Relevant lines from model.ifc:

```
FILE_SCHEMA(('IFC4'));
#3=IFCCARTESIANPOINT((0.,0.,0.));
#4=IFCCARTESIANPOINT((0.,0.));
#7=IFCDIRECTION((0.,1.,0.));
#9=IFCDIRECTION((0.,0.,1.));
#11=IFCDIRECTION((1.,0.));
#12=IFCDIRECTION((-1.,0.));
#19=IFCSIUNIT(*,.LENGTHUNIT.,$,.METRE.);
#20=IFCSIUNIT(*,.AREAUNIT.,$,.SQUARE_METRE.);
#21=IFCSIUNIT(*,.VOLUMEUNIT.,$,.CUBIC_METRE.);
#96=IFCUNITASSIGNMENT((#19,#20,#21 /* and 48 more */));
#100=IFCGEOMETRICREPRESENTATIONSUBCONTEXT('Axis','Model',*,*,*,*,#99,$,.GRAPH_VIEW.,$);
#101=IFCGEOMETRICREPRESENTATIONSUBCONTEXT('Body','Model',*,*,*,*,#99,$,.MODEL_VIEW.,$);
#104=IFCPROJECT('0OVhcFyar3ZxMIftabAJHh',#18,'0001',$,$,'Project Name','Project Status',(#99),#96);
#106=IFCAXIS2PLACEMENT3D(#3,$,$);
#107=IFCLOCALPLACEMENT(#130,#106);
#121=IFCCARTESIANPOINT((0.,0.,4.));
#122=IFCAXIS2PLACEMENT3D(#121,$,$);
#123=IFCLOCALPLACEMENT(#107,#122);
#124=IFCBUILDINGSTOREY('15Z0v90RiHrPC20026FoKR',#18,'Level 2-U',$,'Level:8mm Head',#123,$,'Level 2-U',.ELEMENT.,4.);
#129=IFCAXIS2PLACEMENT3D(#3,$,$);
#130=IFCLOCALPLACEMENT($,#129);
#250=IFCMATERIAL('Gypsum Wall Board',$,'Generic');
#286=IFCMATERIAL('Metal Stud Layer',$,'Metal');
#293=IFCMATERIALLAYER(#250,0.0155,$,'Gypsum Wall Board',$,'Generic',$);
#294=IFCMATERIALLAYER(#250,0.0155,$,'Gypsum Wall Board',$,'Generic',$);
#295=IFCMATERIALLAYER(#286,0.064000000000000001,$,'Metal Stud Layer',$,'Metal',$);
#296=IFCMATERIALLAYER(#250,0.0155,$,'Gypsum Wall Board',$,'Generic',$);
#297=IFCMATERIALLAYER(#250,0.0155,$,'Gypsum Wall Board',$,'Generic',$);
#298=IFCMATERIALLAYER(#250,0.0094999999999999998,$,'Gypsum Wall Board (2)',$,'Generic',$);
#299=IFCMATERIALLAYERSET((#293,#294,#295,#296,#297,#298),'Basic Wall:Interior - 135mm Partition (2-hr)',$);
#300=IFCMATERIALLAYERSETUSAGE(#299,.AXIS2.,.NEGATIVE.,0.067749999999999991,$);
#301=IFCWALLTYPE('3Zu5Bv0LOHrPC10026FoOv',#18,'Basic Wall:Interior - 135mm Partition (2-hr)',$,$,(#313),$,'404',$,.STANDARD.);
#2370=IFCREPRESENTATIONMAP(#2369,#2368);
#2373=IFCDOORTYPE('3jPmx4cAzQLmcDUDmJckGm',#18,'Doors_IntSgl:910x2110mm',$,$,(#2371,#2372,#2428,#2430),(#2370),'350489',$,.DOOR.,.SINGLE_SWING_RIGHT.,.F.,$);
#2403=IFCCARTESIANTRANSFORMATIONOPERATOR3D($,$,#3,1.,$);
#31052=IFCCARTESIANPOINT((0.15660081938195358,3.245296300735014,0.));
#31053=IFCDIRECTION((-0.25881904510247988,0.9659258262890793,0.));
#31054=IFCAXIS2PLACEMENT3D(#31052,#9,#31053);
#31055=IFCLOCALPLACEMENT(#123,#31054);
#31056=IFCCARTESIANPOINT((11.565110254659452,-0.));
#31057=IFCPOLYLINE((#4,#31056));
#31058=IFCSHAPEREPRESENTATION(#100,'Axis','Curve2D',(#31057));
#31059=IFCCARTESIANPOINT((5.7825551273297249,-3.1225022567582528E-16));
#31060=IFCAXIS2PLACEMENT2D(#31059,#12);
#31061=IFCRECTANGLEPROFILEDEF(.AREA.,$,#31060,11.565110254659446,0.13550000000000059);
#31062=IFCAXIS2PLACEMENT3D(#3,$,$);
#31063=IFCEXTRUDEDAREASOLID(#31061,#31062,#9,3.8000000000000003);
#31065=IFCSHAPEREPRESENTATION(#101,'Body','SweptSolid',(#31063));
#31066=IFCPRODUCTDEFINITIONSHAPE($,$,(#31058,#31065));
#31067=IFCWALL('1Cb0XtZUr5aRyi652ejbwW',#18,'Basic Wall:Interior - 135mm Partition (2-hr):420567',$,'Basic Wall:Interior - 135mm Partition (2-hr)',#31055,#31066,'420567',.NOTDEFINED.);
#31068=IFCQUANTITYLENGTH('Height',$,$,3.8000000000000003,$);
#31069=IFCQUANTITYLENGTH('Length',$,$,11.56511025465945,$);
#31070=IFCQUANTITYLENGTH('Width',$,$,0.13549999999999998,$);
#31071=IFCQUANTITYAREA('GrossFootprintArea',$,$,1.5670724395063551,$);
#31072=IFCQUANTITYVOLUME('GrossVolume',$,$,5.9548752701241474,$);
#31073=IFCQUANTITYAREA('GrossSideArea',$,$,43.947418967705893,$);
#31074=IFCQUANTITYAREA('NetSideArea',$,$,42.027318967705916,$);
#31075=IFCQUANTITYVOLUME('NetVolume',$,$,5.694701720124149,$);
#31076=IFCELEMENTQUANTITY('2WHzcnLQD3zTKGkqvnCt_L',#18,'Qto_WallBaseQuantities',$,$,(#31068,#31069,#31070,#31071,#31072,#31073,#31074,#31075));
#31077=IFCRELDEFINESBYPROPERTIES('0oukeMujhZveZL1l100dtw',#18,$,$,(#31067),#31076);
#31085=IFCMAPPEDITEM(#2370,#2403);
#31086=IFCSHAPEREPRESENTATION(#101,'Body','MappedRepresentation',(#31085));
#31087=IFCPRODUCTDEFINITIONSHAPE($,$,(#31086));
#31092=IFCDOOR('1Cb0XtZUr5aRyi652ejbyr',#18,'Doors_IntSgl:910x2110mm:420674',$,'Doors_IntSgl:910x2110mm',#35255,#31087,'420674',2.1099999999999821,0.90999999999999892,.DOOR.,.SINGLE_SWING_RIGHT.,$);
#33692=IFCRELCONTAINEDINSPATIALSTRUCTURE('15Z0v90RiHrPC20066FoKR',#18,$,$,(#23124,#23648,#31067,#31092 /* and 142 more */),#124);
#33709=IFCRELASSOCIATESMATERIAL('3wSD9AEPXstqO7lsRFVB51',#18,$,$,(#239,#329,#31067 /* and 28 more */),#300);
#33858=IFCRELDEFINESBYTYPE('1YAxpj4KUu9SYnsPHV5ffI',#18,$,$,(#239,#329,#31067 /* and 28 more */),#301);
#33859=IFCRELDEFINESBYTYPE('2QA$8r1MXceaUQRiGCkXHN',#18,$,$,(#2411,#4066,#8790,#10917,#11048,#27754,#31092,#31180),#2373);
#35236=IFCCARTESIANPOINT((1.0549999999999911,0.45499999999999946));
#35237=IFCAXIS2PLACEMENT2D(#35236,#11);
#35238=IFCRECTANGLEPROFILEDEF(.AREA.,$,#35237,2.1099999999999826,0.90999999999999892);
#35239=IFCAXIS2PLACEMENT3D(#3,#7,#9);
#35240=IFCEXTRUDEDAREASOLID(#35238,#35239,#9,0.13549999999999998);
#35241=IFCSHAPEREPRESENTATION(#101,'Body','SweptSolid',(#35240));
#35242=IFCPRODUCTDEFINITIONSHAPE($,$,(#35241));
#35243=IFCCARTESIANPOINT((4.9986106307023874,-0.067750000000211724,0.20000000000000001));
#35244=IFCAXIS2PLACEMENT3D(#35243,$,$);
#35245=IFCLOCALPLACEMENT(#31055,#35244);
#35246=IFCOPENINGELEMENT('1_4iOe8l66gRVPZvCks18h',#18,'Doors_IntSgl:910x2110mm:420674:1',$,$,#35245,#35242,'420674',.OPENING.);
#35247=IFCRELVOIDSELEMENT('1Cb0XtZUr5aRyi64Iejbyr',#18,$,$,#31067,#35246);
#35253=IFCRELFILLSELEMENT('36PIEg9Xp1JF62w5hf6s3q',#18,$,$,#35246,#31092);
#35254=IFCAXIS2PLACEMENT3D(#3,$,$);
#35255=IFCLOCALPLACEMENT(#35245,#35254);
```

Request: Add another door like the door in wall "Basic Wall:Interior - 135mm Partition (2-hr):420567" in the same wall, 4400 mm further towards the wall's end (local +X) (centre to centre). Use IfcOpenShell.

```python
import ifcopenshell
import ifcopenshell.api.feature
import ifcopenshell.api.geometry
import ifcopenshell.api.pset
import ifcopenshell.api.root
import ifcopenshell.geom
import ifcopenshell.util.element
import ifcopenshell.util.placement
import ifcopenshell.util.shape
import ifcopenshell.util.unit

model = ifcopenshell.open("model.ifc")
area_scale = ifcopenshell.util.unit.calculate_unit_scale(model, "AREAUNIT")
volume_scale = ifcopenshell.util.unit.calculate_unit_scale(model, "VOLUMEUNIT")
settings = ifcopenshell.geom.settings()


def volume(element):
    """Net volume in cubic metres, openings subtracted."""
    shape = ifcopenshell.geom.create_shape(settings, element)
    return ifcopenshell.util.shape.get_volume(shape.geometry)


def reuse_history(source, copy):
    """copy_class also copies each property set's owner history, people and application; keep the originals."""
    for rel in copy.IsDefinedBy:
        if rel.is_a("IfcRelDefinesByProperties") and (history := rel.RelatingPropertyDefinition.OwnerHistory):
            rel.RelatingPropertyDefinition.OwnerHistory = source.OwnerHistory
            ifcopenshell.util.element.remove_deep2(model, history)


door = model.by_id(31092)
opening = door.FillsVoids[0].RelatingOpeningElement
wall = opening.VoidsElements[0].RelatingBuildingElement
before = volume(wall)
shift = ifcopenshell.util.placement.get_local_placement(wall.ObjectPlacement)[:3, 0] * 4.4

# copy_class copies the void relationship, type, container and properties, but no geometry.
new_opening = ifcopenshell.api.root.copy_class(model, product=opening)
new_opening.Representation = ifcopenshell.util.element.copy_deep(
    model, opening.Representation, exclude=["IfcGeometricRepresentationContext", "IfcRepresentationMap"]
)
new_opening.Name = "Doors_IntSgl:910x2110mm"
new_opening.Tag = None
reuse_history(opening, new_opening)
new_door = ifcopenshell.api.root.copy_class(model, product=door)
new_door.Representation = ifcopenshell.util.element.copy_deep(
    model, door.Representation, exclude=["IfcGeometricRepresentationContext", "IfcRepresentationMap"]
)
new_door.Name = "Doors_IntSgl:910x2110mm"
new_door.Tag = None
reuse_history(door, new_door)
ifcopenshell.api.feature.add_filling(model, opening=new_opening, element=new_door)

for old, new in ((opening, new_opening), (door, new_door)):
    matrix = ifcopenshell.util.placement.get_local_placement(old.ObjectPlacement)
    matrix[:3, 3] += shift
    ifcopenshell.api.geometry.edit_object_placement(model, product=new, matrix=matrix, is_si=False)

after = volume(wall)
thickness = 0.1355  # wall thickness in metres

# Update the wall's stored quantities.
qto = model.by_id(ifcopenshell.util.element.get_pset(wall, "Qto_WallBaseQuantities", should_inherit=False)["id"])
ifcopenshell.api.pset.edit_qto(model, qto=qto, properties={
    "NetSideArea": after / thickness / area_scale,
    "NetVolume": after / volume_scale,
})

print(f"wall volume {before:.3f} -> {after:.3f} m3")

model.write("model_edited.ifc")
```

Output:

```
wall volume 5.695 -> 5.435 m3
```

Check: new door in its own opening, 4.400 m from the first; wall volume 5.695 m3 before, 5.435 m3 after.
